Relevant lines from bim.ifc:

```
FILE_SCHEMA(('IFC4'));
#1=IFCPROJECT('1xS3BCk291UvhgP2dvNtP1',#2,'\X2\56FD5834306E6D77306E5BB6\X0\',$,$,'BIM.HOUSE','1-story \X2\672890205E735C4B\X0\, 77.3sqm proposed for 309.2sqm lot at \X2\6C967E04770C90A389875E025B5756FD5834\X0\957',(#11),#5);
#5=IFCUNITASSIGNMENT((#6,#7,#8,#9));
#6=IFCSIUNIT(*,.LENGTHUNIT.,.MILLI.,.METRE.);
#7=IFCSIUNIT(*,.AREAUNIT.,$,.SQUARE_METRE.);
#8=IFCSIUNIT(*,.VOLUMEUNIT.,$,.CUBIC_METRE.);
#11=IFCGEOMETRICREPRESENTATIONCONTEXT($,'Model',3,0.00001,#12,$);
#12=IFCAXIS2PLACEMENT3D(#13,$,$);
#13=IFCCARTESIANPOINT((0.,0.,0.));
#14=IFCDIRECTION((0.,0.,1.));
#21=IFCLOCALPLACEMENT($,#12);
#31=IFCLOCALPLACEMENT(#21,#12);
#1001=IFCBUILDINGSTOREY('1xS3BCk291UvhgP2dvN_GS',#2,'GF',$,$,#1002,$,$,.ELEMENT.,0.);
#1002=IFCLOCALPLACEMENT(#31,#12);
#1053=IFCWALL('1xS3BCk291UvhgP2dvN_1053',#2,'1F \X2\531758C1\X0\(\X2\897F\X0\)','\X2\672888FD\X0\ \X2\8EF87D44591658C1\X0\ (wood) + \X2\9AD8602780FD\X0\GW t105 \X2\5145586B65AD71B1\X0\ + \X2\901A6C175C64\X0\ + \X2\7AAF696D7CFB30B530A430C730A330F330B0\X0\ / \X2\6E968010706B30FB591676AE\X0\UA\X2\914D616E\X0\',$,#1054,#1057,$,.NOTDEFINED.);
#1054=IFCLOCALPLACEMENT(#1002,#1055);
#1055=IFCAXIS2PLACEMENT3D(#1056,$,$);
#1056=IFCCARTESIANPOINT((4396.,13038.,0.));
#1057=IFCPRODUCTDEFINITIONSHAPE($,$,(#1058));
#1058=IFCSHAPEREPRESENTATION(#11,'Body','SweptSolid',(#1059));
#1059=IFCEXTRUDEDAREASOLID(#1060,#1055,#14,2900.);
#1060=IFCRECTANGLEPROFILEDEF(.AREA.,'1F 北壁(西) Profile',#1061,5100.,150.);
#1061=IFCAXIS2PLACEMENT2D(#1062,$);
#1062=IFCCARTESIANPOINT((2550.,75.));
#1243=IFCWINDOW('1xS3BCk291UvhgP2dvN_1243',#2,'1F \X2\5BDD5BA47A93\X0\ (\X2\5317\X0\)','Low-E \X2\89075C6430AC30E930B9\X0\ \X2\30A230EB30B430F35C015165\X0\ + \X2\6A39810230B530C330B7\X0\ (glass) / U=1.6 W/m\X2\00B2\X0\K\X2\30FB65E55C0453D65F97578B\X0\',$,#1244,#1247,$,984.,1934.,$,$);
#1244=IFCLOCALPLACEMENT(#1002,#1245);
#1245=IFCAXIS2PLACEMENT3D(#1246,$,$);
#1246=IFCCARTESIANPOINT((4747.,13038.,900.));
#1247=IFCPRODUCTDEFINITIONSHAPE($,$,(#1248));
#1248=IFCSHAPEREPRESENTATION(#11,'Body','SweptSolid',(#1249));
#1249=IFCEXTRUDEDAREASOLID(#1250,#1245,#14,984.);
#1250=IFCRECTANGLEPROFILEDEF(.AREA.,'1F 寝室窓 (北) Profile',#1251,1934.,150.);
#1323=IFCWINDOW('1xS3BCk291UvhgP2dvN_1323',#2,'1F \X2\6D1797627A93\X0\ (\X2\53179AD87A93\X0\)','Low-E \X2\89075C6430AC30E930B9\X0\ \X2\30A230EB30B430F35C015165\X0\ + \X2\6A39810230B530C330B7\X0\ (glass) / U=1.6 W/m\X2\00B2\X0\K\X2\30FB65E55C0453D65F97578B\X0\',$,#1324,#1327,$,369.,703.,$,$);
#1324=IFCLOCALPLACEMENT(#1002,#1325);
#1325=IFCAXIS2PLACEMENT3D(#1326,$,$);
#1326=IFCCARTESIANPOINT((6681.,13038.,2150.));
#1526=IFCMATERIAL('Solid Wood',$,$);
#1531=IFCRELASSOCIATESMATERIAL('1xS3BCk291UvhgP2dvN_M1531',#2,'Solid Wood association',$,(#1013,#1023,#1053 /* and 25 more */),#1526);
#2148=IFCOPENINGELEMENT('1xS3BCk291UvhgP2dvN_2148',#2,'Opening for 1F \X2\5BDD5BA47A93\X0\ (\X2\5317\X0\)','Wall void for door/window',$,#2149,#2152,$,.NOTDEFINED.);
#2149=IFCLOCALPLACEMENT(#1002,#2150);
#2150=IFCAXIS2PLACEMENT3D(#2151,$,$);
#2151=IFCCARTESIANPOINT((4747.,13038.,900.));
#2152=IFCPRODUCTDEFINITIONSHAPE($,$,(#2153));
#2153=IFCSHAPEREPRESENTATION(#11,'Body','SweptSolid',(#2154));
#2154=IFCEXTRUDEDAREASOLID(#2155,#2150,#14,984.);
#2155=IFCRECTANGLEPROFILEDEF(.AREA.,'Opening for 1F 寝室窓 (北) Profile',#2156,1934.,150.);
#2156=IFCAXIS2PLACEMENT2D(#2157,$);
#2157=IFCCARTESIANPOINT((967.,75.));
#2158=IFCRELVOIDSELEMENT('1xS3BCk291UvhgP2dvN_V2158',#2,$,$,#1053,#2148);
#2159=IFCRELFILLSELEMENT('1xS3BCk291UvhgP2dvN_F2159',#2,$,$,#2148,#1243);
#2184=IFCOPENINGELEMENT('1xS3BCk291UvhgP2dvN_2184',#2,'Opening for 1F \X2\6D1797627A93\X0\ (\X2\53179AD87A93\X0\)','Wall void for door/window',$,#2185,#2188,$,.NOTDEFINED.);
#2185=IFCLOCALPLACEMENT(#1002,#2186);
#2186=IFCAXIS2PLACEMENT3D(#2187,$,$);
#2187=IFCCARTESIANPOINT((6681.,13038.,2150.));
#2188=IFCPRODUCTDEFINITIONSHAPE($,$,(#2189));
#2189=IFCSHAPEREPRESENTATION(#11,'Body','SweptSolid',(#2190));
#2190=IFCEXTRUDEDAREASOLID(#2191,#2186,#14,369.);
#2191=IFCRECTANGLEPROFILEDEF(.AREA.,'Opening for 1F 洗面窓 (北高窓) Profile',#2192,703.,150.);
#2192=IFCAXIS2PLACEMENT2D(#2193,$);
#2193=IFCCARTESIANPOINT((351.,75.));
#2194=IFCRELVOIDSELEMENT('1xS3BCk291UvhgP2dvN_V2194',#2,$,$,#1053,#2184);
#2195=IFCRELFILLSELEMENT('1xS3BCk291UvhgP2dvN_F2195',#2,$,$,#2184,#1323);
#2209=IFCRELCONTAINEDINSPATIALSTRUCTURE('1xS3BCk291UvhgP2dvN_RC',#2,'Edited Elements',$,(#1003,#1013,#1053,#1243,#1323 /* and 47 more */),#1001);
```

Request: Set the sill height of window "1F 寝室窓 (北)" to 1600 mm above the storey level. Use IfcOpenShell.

```python
import numpy as np
import ifcopenshell
import ifcopenshell.api.geometry
import ifcopenshell.geom
import ifcopenshell.util.element
import ifcopenshell.util.placement
import ifcopenshell.util.shape
import ifcopenshell.util.unit

model = ifcopenshell.open("bim.ifc")
unit_scale = ifcopenshell.util.unit.calculate_unit_scale(model)

window = model.by_guid("1xS3BCk291UvhgP2dvN_1243")
opening = window.FillsVoids[0].RelatingOpeningElement
storey = ifcopenshell.util.element.get_container(window, ifc_class="IfcBuildingStorey")
level = ifcopenshell.util.placement.get_local_placement(storey.ObjectPlacement)[2, 3]

# The opening's origin need not be at the sill, so measure its lowest point.
shape = ifcopenshell.geom.create_shape(ifcopenshell.geom.settings(), opening)
bottom = ifcopenshell.util.shape.get_shape_bottom_elevation(shape, shape.geometry) / unit_scale
dz = level + 1.6 / unit_scale - bottom

shift = np.array([0.0, 0.0, dz])
# The window is not placed relative to its opening, so move both.
for product in (opening, window):
    matrix = ifcopenshell.util.placement.get_local_placement(product.ObjectPlacement)
    matrix[:3, 3] += shift
    ifcopenshell.api.geometry.edit_object_placement(model, product=product, matrix=matrix, is_si=False)

print(f"moved by {dz * unit_scale:+.3f} m")

model.write("bim_edited.ifc")
```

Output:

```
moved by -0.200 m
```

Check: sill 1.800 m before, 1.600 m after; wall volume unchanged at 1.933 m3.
